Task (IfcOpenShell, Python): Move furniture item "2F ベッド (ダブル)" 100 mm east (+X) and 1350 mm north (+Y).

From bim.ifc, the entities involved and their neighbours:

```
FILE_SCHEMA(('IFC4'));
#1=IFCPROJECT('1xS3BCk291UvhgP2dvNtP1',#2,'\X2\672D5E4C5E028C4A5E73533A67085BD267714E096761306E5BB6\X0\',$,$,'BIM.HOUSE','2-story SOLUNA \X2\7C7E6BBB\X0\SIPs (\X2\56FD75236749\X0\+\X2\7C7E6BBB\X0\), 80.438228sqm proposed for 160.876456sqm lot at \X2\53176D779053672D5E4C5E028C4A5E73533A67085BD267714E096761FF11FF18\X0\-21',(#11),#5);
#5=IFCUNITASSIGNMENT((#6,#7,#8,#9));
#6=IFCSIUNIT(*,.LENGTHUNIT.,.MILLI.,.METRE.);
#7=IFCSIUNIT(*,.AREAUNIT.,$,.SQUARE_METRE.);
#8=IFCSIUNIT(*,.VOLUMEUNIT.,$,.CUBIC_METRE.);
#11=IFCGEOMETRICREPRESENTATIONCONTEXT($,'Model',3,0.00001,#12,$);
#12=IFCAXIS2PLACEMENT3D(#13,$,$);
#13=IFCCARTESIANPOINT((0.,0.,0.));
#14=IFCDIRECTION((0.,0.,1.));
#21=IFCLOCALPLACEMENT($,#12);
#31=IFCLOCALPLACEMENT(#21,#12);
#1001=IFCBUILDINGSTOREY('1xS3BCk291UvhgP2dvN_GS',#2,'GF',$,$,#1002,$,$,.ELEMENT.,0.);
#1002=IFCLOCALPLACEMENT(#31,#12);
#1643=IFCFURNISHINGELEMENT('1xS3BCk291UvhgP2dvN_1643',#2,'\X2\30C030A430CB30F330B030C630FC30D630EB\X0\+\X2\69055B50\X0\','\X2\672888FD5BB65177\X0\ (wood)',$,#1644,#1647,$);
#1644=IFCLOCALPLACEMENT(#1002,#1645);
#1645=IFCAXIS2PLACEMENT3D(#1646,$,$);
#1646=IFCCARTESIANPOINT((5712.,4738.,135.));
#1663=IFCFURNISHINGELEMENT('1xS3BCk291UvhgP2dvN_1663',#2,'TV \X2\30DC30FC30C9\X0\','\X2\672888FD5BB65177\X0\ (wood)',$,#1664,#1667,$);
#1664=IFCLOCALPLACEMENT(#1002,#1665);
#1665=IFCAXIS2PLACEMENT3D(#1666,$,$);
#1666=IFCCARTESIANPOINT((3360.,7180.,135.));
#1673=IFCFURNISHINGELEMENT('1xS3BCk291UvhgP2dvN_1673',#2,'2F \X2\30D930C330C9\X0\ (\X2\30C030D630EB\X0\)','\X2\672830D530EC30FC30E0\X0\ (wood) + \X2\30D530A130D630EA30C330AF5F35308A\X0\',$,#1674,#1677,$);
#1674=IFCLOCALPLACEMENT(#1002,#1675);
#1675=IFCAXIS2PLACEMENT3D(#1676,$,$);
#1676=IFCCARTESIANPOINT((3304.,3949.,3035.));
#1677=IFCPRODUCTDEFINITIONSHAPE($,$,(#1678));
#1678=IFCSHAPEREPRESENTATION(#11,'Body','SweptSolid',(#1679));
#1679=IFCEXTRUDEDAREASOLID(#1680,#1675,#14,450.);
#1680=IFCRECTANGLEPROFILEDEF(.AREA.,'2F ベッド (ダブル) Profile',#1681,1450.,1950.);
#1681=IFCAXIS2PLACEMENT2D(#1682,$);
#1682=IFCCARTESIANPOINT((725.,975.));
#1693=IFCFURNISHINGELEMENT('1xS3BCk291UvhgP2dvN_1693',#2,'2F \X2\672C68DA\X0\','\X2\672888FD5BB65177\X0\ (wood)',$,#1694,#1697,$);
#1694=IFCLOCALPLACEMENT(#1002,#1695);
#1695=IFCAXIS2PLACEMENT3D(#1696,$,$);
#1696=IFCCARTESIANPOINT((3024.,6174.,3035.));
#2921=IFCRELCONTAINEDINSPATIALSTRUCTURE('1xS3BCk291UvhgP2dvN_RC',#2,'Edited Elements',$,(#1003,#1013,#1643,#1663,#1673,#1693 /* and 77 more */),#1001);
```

```python
import ifcopenshell
import ifcopenshell.api.geometry
import ifcopenshell.util.placement

model = ifcopenshell.open("bim.ifc")

item = model.by_guid("1xS3BCk291UvhgP2dvN_1673")
matrix = ifcopenshell.util.placement.get_local_placement(item.ObjectPlacement)
matrix[0, 3] += 100.0
matrix[1, 3] += 1350.0
ifcopenshell.api.geometry.edit_object_placement(model, product=item, matrix=matrix, is_si=False)

print(ifcopenshell.util.placement.get_local_placement(item.ObjectPlacement).round(3) + 0.0)

model.write("bim_updated.ifc")
```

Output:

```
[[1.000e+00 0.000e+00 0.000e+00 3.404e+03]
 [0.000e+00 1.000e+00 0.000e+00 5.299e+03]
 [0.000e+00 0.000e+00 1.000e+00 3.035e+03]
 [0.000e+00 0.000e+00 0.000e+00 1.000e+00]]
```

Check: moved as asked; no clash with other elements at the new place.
